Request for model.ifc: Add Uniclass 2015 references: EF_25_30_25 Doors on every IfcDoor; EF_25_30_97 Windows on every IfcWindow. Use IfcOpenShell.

First a look at what the model holds.

```python
import ifcopenshell

model = ifcopenshell.open("model.ifc")
print(model.schema)
print("classifications:", [c.Name for c in model.by_type("IfcClassification")])
for ifc_class in ("IfcDoor", "IfcRoof", "IfcStair", "IfcWall", "IfcWindow"):
    print(ifc_class, len(model.by_type(ifc_class)))
```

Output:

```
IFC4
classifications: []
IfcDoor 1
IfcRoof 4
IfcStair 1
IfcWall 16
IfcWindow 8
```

```python
import ifcopenshell
import ifcopenshell.api.classification

model = ifcopenshell.open("model.ifc")

system = ifcopenshell.api.classification.add_classification(model, classification="Uniclass 2015")

codes = {
    "IfcDoor": ("EF_25_30_25", "Doors"),
    "IfcWindow": ("EF_25_30_97", "Windows"),
}
for ifc_class, (code, name) in codes.items():
    products = model.by_type(ifc_class)
    ifcopenshell.api.classification.add_reference(
        model, products=products, classification=system, identification=code, name=name
    )
    print(code, len(products))

model.write("model_v2.ifc")
```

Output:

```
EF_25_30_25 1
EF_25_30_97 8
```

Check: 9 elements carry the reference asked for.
